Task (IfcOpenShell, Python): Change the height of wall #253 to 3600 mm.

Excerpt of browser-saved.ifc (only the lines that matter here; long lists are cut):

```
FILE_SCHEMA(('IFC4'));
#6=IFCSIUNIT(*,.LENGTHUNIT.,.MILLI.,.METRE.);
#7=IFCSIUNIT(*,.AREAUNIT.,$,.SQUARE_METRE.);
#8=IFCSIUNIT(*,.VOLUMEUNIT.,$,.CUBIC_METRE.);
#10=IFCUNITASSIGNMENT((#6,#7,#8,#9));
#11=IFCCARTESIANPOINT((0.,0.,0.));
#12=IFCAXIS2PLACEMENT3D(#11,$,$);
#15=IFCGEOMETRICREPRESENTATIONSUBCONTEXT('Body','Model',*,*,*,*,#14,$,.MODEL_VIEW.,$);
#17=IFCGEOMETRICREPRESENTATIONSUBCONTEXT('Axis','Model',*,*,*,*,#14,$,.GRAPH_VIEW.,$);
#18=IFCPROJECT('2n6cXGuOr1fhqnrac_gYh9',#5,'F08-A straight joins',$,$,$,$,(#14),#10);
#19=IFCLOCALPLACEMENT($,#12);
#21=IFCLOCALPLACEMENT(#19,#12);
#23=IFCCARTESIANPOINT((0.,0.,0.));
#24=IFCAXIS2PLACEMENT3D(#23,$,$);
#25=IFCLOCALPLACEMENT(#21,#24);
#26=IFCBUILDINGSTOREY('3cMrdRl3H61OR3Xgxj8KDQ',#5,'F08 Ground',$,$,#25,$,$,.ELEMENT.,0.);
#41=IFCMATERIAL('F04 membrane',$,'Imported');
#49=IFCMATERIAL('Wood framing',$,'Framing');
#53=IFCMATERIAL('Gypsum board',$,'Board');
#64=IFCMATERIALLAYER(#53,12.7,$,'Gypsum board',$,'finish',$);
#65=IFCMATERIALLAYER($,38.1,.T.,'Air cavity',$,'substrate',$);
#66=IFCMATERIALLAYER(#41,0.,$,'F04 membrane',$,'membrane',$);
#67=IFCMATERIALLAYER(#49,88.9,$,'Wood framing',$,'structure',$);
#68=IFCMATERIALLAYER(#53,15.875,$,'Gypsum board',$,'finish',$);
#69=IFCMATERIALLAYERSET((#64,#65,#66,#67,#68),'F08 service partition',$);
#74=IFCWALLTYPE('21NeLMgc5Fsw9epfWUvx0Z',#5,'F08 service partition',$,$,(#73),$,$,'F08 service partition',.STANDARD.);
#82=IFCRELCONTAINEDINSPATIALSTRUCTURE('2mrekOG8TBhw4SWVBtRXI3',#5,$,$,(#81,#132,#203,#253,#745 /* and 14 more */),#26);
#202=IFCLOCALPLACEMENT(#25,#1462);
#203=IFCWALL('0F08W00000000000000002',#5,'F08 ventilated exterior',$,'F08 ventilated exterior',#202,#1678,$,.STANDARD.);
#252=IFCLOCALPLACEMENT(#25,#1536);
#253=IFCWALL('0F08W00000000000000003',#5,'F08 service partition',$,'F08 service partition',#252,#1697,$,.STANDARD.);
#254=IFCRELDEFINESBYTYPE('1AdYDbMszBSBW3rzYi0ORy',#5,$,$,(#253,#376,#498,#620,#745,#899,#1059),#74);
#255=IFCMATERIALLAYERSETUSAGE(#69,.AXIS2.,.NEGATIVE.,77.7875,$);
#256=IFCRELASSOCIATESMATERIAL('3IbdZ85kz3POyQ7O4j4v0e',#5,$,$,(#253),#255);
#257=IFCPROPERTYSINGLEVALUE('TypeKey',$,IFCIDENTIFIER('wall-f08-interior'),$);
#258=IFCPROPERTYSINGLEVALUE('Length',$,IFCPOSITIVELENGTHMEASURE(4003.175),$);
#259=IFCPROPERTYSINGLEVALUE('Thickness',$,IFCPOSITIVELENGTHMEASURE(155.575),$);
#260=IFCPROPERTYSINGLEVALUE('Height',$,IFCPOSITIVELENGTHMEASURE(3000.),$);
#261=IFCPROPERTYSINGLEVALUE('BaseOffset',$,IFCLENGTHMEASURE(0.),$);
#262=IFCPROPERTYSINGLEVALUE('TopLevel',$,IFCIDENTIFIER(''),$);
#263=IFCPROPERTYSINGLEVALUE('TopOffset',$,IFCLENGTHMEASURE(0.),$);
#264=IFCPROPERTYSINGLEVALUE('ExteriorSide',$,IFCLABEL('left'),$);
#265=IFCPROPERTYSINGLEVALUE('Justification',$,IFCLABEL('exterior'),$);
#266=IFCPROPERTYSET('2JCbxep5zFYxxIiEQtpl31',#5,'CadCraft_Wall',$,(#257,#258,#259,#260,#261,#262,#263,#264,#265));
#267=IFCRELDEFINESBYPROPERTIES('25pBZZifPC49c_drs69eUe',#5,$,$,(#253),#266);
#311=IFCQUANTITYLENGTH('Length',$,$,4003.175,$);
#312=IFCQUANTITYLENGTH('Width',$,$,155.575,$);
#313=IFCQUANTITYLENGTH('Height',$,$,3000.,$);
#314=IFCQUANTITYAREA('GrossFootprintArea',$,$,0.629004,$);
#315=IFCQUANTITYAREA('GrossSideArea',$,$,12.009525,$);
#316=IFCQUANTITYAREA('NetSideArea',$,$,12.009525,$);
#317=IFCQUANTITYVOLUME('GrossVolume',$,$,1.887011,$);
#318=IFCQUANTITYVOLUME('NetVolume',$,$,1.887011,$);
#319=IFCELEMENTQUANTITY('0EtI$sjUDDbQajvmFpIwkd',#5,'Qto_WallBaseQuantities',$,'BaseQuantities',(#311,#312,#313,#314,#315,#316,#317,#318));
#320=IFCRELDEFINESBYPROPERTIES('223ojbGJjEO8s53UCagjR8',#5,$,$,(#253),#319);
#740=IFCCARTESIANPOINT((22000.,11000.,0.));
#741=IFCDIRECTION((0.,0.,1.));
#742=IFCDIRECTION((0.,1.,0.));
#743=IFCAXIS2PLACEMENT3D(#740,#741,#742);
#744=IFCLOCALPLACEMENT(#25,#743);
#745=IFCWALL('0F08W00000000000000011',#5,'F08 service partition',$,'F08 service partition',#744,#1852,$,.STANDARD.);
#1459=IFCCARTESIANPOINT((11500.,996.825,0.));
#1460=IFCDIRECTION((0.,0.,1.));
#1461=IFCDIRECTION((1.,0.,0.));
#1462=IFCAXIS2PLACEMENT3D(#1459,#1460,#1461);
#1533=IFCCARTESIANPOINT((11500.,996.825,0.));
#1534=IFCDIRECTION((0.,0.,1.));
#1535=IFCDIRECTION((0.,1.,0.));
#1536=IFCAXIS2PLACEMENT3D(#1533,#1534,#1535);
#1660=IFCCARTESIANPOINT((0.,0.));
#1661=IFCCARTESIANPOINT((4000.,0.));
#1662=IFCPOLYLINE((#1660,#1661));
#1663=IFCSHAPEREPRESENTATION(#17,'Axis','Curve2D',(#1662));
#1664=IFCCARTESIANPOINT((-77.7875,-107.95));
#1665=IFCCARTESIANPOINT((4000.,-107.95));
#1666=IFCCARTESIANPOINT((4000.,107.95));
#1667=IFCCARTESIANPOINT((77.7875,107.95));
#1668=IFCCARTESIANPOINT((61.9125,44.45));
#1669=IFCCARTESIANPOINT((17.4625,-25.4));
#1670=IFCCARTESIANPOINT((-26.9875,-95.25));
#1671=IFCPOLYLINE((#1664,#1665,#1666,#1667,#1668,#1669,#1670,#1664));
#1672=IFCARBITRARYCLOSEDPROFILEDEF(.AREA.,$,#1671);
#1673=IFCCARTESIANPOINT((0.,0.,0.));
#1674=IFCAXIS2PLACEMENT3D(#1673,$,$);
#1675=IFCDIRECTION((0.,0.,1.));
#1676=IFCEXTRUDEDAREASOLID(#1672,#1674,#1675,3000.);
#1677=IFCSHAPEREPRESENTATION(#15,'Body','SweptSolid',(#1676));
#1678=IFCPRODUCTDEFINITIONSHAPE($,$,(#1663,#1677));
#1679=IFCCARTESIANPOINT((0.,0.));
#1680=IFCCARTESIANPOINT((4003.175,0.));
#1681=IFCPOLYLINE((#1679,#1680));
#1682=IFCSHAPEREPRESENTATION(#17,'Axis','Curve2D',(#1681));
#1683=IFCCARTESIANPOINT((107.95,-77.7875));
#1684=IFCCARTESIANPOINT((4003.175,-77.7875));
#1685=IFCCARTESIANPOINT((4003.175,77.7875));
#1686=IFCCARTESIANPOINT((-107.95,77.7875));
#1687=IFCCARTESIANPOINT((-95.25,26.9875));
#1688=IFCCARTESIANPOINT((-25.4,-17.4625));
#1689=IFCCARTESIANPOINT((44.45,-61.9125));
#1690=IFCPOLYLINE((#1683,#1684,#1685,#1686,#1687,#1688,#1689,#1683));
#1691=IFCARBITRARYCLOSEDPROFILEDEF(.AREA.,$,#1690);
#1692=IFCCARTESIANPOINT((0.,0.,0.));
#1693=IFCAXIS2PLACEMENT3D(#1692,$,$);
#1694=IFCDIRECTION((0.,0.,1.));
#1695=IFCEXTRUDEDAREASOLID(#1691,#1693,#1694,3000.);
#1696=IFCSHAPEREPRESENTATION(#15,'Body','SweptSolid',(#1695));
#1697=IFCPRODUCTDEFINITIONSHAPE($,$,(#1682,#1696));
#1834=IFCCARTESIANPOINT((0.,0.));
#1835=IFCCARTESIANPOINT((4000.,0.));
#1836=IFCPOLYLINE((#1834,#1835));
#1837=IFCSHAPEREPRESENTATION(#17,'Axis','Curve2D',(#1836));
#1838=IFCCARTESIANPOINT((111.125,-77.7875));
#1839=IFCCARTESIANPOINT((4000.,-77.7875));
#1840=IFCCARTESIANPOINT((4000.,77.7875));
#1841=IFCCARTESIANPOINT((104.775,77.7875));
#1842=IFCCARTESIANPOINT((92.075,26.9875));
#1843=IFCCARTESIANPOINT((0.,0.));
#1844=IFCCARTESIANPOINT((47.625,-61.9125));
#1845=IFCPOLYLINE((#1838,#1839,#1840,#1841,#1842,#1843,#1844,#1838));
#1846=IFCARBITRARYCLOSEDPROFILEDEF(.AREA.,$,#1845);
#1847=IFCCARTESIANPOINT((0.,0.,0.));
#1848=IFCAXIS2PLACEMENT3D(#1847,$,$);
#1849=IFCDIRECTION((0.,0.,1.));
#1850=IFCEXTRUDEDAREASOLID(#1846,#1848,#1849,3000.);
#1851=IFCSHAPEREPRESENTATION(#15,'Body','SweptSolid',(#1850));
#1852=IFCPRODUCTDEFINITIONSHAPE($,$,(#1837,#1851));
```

```python
import ifcopenshell
import ifcopenshell.api.pset
import ifcopenshell.geom
import ifcopenshell.util.element
import ifcopenshell.util.representation
import ifcopenshell.util.shape
import ifcopenshell.util.unit

model = ifcopenshell.open("browser-saved.ifc")
unit_scale = ifcopenshell.util.unit.calculate_unit_scale(model)
area_scale = ifcopenshell.util.unit.calculate_unit_scale(model, "AREAUNIT")
volume_scale = ifcopenshell.util.unit.calculate_unit_scale(model, "VOLUMEUNIT")
settings = ifcopenshell.geom.settings()


def volume(element):
    """Net volume in cubic metres, openings subtracted."""
    shape = ifcopenshell.geom.create_shape(settings, element)
    return ifcopenshell.util.shape.get_volume(shape.geometry)


wall = model.by_guid("0F08W00000000000000003")
before = volume(wall)

body = ifcopenshell.util.representation.get_representation(wall, "Model", "Body")
solid = body.Items[0]
old_height = solid.Depth
solid.Depth = 3.6 / unit_scale
after = volume(wall)
thickness = 0.1556  # wall thickness in metres

# Update the stored height, areas and volumes.
pset = model.by_id(ifcopenshell.util.element.get_pset(wall, "CadCraft_Wall", should_inherit=False)["id"])
ifcopenshell.api.pset.edit_pset(model, pset=pset, properties={
    "Height": model.create_entity("IfcPositiveLengthMeasure", solid.Depth),
})
qto = model.by_id(ifcopenshell.util.element.get_pset(wall, "Qto_WallBaseQuantities", should_inherit=False)["id"])
ifcopenshell.api.pset.edit_qto(model, qto=qto, properties={
    "Height": solid.Depth,
    "GrossSideArea": ifcopenshell.util.element.get_pset(wall, "Qto_WallBaseQuantities", "GrossSideArea") * solid.Depth / old_height,
    "NetSideArea": after / thickness / area_scale,
    "GrossVolume": ifcopenshell.util.element.get_pset(wall, "Qto_WallBaseQuantities", "GrossVolume") * solid.Depth / old_height,
    "NetVolume": after / volume_scale,
})

print(f"height {old_height:g} -> {solid.Depth:g}, volume {before:.3f} -> {after:.3f} m3")

model.write("browser-saved_v2.ifc")
```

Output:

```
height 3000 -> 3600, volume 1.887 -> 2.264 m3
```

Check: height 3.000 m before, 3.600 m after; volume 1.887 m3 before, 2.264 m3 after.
